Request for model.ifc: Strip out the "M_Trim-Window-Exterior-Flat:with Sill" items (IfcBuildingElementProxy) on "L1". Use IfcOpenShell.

First a look at what the model holds.

```python
import ifcopenshell
import ifcopenshell.util.element

model = ifcopenshell.open("model.ifc")
print(model.schema)
storey = next(s for s in model.by_type("IfcBuildingStorey") if s.Name == "L1")
proxies = [e for e in ifcopenshell.util.element.get_decomposition(storey) if e.is_a("IfcBuildingElementProxy")]
seen = {}
for e in proxies:
    element_type = ifcopenshell.util.element.get_type(e)
    name = element_type.Name if element_type not in (None, e) else None
    seen[name] = seen.get(name, 0) + 1
for name, count in sorted(seen.items(), key=str):
    print(count, "x", name)
```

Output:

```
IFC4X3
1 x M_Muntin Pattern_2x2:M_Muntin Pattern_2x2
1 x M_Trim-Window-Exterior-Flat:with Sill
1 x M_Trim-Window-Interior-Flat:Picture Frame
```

```python
import ifcopenshell
import ifcopenshell.api.root
import ifcopenshell.util.element

model = ifcopenshell.open("model.ifc")

storey = next(s for s in model.by_type("IfcBuildingStorey") if s.Name == "L1")
proxies = [e for e in ifcopenshell.util.element.get_decomposition(storey) if e.is_a("IfcBuildingElementProxy")]
targets = [e for e in proxies if (t := ifcopenshell.util.element.get_type(e)) not in (None, e) and t.Name == "M_Trim-Window-Exterior-Flat:with Sill"]

for e in targets:
    ifcopenshell.api.root.remove_product(model, product=e)
print(len(targets), "removed")

model.write("model_edited.ifc")
```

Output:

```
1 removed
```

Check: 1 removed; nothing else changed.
